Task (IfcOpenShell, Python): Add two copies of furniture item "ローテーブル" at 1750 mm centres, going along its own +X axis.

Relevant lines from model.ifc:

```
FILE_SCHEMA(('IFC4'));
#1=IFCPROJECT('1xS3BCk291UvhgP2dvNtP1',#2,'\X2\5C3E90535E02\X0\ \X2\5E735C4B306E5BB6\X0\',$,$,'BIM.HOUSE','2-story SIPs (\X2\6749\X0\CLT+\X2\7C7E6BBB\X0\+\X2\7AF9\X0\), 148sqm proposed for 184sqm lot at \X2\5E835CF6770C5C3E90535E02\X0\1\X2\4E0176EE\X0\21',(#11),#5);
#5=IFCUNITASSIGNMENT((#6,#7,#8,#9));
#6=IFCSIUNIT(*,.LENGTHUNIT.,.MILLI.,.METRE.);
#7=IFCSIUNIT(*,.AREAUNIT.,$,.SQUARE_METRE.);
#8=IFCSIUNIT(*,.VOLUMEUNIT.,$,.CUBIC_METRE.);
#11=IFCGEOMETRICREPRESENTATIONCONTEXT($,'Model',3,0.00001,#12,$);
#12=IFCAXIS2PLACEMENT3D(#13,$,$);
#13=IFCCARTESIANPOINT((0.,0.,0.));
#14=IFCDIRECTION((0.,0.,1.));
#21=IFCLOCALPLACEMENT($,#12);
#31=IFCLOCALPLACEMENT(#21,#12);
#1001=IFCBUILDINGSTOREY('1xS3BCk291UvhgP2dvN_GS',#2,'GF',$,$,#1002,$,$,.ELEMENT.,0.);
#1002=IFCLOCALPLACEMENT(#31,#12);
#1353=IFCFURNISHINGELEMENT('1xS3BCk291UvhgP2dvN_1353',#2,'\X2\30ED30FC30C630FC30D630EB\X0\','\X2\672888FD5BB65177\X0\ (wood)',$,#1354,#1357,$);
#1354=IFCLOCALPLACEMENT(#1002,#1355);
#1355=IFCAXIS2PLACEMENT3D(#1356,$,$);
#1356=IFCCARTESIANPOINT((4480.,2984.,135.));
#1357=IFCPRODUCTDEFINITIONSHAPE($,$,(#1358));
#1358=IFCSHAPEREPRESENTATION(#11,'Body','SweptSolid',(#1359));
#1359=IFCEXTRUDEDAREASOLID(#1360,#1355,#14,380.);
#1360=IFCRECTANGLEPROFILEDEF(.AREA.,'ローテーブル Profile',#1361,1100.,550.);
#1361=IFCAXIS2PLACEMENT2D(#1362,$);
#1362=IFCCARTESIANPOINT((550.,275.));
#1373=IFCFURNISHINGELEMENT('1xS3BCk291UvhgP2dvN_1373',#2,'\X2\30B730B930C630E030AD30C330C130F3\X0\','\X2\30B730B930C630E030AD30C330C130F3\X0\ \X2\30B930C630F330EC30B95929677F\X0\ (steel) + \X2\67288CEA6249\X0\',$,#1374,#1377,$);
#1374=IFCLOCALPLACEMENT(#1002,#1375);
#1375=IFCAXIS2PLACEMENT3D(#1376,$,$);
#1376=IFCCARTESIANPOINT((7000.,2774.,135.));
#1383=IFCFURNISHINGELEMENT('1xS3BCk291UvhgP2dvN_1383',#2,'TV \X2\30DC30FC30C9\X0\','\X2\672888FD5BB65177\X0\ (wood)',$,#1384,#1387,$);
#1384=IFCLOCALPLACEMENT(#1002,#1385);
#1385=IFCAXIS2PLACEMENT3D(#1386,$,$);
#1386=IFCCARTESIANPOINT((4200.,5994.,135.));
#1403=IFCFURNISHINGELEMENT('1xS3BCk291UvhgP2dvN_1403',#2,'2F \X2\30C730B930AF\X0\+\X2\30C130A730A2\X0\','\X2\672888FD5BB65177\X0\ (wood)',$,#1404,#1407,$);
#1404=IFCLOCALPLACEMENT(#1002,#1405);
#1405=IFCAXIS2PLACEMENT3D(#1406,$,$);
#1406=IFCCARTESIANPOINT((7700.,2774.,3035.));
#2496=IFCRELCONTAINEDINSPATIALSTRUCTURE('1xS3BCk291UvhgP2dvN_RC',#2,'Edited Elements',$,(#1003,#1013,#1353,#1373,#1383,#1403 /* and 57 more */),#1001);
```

```python
import ifcopenshell
import ifcopenshell.api.geometry
import ifcopenshell.api.root
import ifcopenshell.util.element
import ifcopenshell.util.placement
import ifcopenshell.util.unit

model = ifcopenshell.open("model.ifc")
unit_scale = ifcopenshell.util.unit.calculate_unit_scale(model)


def reuse_history(source, copy):
    """copy_class also copies each property set's owner history, people and application; keep the originals."""
    for rel in copy.IsDefinedBy:
        if rel.is_a("IfcRelDefinesByProperties") and (history := rel.RelatingPropertyDefinition.OwnerHistory):
            rel.RelatingPropertyDefinition.OwnerHistory = source.OwnerHistory
            ifcopenshell.util.element.remove_deep2(model, history)


source = model.by_guid("1xS3BCk291UvhgP2dvN_1353")
base = ifcopenshell.util.placement.get_local_placement(source.ObjectPlacement)
step = base[:3, 0] * 1.75 / unit_scale

for i in range(1, 3):
    copy = ifcopenshell.api.root.copy_class(model, product=source)
    copy.Representation = ifcopenshell.util.element.copy_deep(
        model, source.Representation, exclude=["IfcGeometricRepresentationContext", "IfcRepresentationMap"]
    )
    reuse_history(source, copy)
    matrix = base.copy()
    matrix[:3, 3] += i * step
    print("added at", matrix[:3, 3].round(3) + 0.0)
    ifcopenshell.api.geometry.edit_object_placement(model, product=copy, matrix=matrix, is_si=False)

model.write("model-out.ifc")
```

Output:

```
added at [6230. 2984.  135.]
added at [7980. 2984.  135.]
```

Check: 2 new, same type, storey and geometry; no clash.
